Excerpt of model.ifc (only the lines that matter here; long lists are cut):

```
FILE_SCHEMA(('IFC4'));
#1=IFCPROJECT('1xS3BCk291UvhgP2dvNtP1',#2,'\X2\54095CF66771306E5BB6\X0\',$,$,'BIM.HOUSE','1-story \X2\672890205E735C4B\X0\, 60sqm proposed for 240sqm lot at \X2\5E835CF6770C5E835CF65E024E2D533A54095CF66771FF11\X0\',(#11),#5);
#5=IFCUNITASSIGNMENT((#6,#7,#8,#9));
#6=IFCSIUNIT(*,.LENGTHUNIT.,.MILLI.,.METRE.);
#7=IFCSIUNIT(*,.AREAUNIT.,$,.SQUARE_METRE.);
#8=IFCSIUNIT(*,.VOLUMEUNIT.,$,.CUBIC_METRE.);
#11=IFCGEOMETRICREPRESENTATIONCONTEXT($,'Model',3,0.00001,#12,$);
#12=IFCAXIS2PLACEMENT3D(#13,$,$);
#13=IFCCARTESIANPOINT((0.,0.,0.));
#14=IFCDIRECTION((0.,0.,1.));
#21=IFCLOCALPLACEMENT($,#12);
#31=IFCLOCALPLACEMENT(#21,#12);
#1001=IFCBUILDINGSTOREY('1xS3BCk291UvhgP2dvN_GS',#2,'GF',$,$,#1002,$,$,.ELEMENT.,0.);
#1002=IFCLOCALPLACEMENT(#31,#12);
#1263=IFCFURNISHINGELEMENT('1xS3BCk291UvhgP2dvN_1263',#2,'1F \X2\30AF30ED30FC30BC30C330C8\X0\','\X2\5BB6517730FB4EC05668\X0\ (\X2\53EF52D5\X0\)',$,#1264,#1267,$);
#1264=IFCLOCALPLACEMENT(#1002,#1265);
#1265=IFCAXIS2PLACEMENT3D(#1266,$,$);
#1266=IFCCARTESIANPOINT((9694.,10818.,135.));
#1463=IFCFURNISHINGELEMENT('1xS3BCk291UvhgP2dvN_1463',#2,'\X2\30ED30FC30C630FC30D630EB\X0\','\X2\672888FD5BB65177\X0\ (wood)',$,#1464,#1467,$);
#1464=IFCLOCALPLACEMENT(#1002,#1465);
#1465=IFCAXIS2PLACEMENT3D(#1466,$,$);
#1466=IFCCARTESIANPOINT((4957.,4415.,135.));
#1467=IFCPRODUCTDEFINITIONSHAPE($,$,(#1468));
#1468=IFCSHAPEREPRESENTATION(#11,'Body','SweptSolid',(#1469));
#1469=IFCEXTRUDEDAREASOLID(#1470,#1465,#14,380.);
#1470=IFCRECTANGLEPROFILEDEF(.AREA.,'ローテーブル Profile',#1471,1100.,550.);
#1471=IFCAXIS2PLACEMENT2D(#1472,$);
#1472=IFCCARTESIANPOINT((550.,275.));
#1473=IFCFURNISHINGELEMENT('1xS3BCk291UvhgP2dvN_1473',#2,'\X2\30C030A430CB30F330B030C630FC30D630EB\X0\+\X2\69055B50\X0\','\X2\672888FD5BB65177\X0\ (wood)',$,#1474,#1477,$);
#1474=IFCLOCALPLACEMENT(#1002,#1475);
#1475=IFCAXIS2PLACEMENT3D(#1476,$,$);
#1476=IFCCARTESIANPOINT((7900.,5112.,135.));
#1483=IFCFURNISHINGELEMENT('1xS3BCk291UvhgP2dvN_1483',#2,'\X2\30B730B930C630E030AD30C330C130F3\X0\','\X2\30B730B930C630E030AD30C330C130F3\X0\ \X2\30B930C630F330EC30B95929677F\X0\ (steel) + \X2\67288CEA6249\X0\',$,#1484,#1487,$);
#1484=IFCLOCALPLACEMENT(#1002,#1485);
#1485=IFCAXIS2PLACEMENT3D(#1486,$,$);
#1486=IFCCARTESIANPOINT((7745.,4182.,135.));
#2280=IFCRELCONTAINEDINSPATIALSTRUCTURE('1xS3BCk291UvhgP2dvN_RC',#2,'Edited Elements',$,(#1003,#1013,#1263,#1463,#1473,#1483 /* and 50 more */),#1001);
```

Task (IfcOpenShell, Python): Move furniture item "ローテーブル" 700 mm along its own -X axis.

```python
import ifcopenshell
import ifcopenshell.api.geometry
import ifcopenshell.util.placement
import ifcopenshell.util.unit

model = ifcopenshell.open("model.ifc")
unit_scale = ifcopenshell.util.unit.calculate_unit_scale(model)

item = model.by_id(1463)
matrix = ifcopenshell.util.placement.get_local_placement(item.ObjectPlacement)
matrix[:3, 3] -= matrix[:3, 0] * 0.7 / unit_scale
ifcopenshell.api.geometry.edit_object_placement(model, product=item, matrix=matrix, is_si=False)

print(ifcopenshell.util.placement.get_local_placement(item.ObjectPlacement).round(3) + 0.0)

model.write("model_updated.ifc")
```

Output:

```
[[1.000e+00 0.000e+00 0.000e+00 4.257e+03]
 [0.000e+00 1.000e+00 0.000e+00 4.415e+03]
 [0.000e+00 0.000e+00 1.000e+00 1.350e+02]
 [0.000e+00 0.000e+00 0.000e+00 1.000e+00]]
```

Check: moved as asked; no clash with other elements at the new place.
